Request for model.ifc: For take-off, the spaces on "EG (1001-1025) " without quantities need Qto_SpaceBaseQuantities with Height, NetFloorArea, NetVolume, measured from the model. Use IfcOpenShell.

First a look at what the model holds.

```python
import ifcopenshell
import ifcopenshell.util.element
import ifcopenshell.util.unit

model = ifcopenshell.open("model.ifc")
print(model.schema)
for unit_type in ("LENGTHUNIT", "AREAUNIT", "VOLUMEUNIT"):
    print(unit_type, ifcopenshell.util.unit.calculate_unit_scale(model, unit_type))
storey = next(s for s in model.by_type("IfcBuildingStorey") if s.Name == "EG (1001-1025) ")
spaces = [e for e in ifcopenshell.util.element.get_decomposition(storey) if e.is_a("IfcSpace")]
for e in sorted(spaces, key=lambda e: e.id()):
    print(e.id(), e.is_a(), e.Name, list(ifcopenshell.util.element.get_psets(e, qtos_only=True)), sep=" | ")
```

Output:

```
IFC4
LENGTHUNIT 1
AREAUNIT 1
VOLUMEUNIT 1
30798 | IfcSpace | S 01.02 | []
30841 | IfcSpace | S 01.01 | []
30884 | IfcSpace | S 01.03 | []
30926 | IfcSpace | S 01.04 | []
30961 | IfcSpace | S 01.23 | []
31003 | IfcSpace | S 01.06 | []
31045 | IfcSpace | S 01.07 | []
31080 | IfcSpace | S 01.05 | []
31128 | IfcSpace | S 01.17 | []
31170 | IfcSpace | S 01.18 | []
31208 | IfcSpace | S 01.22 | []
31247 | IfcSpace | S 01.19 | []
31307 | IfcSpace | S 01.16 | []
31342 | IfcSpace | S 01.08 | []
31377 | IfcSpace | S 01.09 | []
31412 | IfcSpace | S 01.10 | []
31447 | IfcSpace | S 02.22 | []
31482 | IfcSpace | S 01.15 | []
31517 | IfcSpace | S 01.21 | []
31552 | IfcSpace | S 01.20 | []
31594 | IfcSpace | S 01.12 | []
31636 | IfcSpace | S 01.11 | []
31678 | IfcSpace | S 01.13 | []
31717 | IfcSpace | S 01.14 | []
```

```python
import ifcopenshell
import ifcopenshell.api.pset
import ifcopenshell.geom
import ifcopenshell.util.element
import ifcopenshell.util.shape
import ifcopenshell.util.unit

model = ifcopenshell.open("model.ifc")
unit_scale = ifcopenshell.util.unit.calculate_unit_scale(model)
area_scale = ifcopenshell.util.unit.calculate_unit_scale(model, "AREAUNIT")
volume_scale = ifcopenshell.util.unit.calculate_unit_scale(model, "VOLUMEUNIT")
settings = ifcopenshell.geom.settings()

storey = next(s for s in model.by_type("IfcBuildingStorey") if s.Name == "EG (1001-1025) ")
spaces = [e for e in ifcopenshell.util.element.get_decomposition(storey) if e.is_a("IfcSpace")]

for e in sorted(spaces, key=lambda e: e.id()):
    if ifcopenshell.util.element.get_psets(e, qtos_only=True, should_inherit=False):
        continue
    # Geometry comes back in metres, in the element's own axes.
    shape = ifcopenshell.geom.create_shape(settings, e)
    values = {
        "Height": ifcopenshell.util.shape.get_z(shape.geometry) / unit_scale,
        "NetFloorArea": ifcopenshell.util.shape.get_footprint_area(shape.geometry) / area_scale,
        "NetVolume": ifcopenshell.util.shape.get_volume(shape.geometry) / volume_scale,
    }
    qto = ifcopenshell.api.pset.add_qto(model, product=e, name="Qto_SpaceBaseQuantities")
    ifcopenshell.api.pset.edit_qto(model, qto=qto, properties=values)
    print(e.id(), {k: round(v, 3) for k, v in values.items()})

model.write("model_edited.ifc")
```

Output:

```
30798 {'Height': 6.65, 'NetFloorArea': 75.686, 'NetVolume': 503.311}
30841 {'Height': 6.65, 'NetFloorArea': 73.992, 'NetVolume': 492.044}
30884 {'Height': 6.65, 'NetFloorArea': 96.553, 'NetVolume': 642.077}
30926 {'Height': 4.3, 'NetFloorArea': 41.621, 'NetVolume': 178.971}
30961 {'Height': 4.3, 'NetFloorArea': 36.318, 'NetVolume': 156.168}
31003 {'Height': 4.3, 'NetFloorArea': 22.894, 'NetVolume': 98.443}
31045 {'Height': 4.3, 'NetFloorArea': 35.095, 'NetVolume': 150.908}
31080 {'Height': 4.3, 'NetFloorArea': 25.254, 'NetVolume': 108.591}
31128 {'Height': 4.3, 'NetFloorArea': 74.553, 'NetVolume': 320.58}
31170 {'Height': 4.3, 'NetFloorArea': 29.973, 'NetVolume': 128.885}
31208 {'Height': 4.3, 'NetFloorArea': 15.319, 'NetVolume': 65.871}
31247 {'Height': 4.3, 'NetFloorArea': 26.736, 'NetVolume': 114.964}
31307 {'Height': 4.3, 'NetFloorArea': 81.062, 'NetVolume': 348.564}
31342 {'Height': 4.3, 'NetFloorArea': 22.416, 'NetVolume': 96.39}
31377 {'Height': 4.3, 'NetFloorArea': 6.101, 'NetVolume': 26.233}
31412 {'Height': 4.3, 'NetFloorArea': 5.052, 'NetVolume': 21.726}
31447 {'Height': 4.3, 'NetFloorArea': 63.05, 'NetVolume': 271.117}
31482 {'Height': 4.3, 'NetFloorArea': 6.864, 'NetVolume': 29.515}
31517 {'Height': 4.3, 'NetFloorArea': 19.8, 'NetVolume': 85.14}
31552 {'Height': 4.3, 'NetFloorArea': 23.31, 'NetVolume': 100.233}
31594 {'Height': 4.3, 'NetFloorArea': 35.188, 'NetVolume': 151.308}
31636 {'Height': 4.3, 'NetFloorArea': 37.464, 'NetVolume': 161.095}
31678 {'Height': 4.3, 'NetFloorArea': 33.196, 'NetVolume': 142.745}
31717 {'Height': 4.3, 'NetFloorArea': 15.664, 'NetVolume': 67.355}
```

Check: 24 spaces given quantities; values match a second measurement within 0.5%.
